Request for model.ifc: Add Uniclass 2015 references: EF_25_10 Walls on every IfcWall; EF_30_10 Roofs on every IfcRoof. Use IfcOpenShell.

First a look at what the model holds.

```python
import ifcopenshell

model = ifcopenshell.open("model.ifc")
print(model.schema)
print("classifications:", [c.Name for c in model.by_type("IfcClassification")])
for ifc_class in ("IfcDoor", "IfcRoof", "IfcStair", "IfcWall", "IfcWindow"):
    print(ifc_class, len(model.by_type(ifc_class)))
```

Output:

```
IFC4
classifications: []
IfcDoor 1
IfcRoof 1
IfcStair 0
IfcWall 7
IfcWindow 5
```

```python
import ifcopenshell
import ifcopenshell.api.classification

model = ifcopenshell.open("model.ifc")

system = ifcopenshell.api.classification.add_classification(model, classification="Uniclass 2015")

codes = {
    "IfcWall": ("EF_25_10", "Walls"),
    "IfcRoof": ("EF_30_10", "Roofs"),
}
for ifc_class, (code, name) in codes.items():
    products = model.by_type(ifc_class)
    ifcopenshell.api.classification.add_reference(
        model, products=products, classification=system, identification=code, name=name
    )
    print(code, len(products))

model.write("model_rev.ifc")
```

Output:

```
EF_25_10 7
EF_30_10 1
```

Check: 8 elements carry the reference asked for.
